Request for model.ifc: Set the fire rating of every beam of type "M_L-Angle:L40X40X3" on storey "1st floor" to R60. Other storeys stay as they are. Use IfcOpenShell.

First a look at what the model holds.

```python
import ifcopenshell
import ifcopenshell.util.element

model = ifcopenshell.open("model.ifc")
print(model.schema)
storey = next(s for s in model.by_type("IfcBuildingStorey") if s.Name == "1st floor")
beams = [e for e in ifcopenshell.util.element.get_decomposition(storey) if e.is_a("IfcBeam")]
seen = {}
for e in beams:
    element_type = ifcopenshell.util.element.get_type(e)
    key = (element_type.Name if element_type != e and element_type else None, ifcopenshell.util.element.get_pset(e, "Pset_BeamCommon", "FireRating"))
    seen[key] = seen.get(key, 0) + 1
for (name, value), count in sorted(seen.items(), key=str):
    print(count, "x", name, "|", value)
```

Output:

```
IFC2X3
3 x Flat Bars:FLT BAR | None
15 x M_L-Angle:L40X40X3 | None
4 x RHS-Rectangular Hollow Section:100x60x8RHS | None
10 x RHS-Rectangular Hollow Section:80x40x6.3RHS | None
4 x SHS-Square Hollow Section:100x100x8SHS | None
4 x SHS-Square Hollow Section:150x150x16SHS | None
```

```python
import ifcopenshell
import ifcopenshell.api.pset
import ifcopenshell.util.element

model = ifcopenshell.open("model.ifc")

storey = next(s for s in model.by_type("IfcBuildingStorey") if s.Name == "1st floor")
beams = [e for e in ifcopenshell.util.element.get_decomposition(storey) if e.is_a("IfcBeam")]

count = 0
for e in beams:
    element_type = ifcopenshell.util.element.get_type(e)
    if element_type in (None, e) or element_type.Name != "M_L-Angle:L40X40X3":
        continue
    # add_pset returns the element's existing set when there is one.
    pset = ifcopenshell.api.pset.add_pset(model, product=e, name="Pset_BeamCommon")
    ifcopenshell.api.pset.edit_pset(model, pset=pset, properties={"FireRating": "R60"})
    count += 1

print(count, "beams updated")

model.write("model_rev.ifc")
```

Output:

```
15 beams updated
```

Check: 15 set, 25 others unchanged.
